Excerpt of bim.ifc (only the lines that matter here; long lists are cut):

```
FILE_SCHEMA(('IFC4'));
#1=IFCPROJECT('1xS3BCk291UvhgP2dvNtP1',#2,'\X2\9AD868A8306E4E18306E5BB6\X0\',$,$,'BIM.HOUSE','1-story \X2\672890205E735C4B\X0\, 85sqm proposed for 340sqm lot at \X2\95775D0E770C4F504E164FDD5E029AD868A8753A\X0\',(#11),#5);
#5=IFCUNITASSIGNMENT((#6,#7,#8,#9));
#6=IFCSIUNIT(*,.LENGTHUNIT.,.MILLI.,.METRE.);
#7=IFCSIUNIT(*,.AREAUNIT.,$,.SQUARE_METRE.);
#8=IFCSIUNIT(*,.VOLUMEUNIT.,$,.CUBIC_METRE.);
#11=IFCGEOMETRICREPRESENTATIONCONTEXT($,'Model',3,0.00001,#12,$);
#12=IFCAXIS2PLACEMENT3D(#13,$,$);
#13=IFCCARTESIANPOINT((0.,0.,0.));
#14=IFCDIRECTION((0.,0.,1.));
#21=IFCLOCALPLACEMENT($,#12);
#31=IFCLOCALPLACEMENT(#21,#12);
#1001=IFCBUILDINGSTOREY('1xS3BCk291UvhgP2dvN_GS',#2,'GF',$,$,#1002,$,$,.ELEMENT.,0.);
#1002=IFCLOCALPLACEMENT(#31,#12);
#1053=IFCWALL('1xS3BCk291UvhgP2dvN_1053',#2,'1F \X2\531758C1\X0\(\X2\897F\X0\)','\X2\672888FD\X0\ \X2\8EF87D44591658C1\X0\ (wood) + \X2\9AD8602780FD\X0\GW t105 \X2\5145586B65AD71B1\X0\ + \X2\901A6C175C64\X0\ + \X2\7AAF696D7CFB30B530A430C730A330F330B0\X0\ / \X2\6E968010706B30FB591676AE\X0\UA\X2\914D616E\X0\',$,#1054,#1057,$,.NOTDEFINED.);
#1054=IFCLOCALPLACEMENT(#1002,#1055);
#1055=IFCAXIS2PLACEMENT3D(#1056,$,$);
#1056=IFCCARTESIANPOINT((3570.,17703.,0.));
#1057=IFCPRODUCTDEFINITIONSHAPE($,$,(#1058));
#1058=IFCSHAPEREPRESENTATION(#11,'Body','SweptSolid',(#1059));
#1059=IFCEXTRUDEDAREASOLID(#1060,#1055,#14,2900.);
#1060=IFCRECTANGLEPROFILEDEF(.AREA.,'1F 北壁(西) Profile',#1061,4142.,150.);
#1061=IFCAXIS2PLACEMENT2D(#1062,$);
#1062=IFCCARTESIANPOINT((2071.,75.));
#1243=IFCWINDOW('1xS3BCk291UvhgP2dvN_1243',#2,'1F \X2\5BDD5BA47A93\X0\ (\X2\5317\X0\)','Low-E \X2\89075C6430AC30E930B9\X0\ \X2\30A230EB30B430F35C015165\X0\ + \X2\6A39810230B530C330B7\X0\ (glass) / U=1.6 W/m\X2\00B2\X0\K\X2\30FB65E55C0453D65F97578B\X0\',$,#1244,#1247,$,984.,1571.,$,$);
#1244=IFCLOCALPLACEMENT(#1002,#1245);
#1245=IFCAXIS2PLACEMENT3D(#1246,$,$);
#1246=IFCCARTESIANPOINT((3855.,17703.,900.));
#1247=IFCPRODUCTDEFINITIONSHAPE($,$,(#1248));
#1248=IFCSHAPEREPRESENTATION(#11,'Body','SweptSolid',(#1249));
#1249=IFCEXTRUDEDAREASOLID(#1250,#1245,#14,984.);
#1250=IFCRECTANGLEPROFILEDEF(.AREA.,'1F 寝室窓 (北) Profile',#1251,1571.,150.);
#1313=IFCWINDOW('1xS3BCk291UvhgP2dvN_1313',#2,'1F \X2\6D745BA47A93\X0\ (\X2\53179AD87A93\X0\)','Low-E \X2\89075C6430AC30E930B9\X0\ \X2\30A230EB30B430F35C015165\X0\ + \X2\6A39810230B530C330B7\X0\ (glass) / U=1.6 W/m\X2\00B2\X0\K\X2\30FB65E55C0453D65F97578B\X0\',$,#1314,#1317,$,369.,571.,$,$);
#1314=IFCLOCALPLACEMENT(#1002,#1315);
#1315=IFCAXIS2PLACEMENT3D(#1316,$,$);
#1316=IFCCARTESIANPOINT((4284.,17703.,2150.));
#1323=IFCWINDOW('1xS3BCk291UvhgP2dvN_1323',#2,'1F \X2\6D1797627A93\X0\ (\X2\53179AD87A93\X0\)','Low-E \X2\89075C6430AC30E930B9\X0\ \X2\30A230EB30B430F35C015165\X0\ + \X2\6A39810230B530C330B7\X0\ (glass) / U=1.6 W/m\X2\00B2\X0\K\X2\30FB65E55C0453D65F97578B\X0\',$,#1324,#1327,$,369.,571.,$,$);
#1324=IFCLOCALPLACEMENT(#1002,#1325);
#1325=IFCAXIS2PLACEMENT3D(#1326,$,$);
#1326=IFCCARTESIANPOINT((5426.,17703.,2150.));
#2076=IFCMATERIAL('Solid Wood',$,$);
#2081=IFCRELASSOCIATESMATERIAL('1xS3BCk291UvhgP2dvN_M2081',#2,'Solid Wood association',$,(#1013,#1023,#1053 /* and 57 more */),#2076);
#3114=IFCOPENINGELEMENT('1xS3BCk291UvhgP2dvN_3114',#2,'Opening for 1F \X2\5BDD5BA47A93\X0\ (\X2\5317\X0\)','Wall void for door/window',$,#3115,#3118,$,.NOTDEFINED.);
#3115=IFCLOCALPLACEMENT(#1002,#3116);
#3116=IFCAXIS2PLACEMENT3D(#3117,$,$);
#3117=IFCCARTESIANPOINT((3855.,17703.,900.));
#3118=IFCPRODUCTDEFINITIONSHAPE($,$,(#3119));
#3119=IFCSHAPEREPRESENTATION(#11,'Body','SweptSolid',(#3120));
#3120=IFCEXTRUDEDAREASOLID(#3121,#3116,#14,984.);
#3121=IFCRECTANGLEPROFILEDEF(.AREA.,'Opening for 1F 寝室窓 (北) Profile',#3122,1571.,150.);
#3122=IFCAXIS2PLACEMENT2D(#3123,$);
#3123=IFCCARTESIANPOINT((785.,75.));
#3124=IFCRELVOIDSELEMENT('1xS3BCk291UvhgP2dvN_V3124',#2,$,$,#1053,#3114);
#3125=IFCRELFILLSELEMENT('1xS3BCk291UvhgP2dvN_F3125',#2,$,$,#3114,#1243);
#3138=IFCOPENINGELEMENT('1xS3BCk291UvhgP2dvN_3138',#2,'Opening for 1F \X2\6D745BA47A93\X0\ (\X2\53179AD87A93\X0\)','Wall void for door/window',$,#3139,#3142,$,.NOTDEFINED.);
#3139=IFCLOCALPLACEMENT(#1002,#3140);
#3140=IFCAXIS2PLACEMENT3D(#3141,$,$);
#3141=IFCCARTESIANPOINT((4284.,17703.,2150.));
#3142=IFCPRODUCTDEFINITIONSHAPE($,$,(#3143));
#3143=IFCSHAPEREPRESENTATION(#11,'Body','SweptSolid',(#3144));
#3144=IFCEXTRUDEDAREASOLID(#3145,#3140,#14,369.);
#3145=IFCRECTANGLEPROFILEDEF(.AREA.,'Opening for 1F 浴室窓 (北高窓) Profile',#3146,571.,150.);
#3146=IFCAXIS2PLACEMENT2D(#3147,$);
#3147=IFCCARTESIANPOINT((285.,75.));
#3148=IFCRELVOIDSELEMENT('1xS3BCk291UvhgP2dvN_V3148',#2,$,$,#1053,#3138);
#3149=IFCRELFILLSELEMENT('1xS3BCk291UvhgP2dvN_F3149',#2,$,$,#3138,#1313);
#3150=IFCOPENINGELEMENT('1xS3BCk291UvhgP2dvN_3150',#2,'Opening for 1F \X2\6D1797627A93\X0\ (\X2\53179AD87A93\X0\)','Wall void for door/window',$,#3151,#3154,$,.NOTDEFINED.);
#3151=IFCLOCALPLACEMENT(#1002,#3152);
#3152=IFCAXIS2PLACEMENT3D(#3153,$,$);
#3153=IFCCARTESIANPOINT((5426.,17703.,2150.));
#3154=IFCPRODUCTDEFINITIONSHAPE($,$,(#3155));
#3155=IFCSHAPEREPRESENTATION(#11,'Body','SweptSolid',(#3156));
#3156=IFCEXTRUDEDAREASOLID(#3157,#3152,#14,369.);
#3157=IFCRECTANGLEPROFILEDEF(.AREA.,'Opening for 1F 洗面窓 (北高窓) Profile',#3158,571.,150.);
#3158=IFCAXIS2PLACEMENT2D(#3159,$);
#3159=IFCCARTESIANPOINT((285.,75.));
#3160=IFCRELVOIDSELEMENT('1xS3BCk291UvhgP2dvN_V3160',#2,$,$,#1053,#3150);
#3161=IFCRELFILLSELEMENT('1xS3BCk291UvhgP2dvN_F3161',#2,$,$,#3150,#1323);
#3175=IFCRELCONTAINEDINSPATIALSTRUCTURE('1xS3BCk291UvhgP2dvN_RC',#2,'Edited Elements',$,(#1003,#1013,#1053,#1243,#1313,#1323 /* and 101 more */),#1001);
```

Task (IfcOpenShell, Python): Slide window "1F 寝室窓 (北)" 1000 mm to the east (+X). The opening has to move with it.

```python
import ifcopenshell
import ifcopenshell.api.geometry
import ifcopenshell.util.placement

model = ifcopenshell.open("bim.ifc")

window = model.by_guid("1xS3BCk291UvhgP2dvN_1243")
opening = window.FillsVoids[0].RelatingOpeningElement
wall = opening.VoidsElements[0].RelatingBuildingElement

wall_matrix = ifcopenshell.util.placement.get_local_placement(wall.ObjectPlacement)
shift = wall_matrix[:3, 0] * 1000.0
before = ifcopenshell.util.placement.get_local_placement(window.ObjectPlacement)[:3, 3].copy()

# The window is not placed relative to its opening, so move both.
for product in (opening, window):
    matrix = ifcopenshell.util.placement.get_local_placement(product.ObjectPlacement)
    matrix[:3, 3] += shift
    ifcopenshell.api.geometry.edit_object_placement(model, product=product, matrix=matrix, is_si=False)

after = ifcopenshell.util.placement.get_local_placement(window.ObjectPlacement)[:3, 3]
print("window moved by", (after - before).round(3) + 0.0)

model.write("bim_v2.ifc")
```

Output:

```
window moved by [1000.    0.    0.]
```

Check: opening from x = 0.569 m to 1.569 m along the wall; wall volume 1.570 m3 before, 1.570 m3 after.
